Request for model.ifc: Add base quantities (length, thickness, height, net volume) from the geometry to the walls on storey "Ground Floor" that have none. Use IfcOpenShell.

First a look at what the model holds.

```python
import ifcopenshell
import ifcopenshell.util.element
import ifcopenshell.util.unit

model = ifcopenshell.open("model.ifc")
print(model.schema)
for unit_type in ("LENGTHUNIT", "AREAUNIT", "VOLUMEUNIT"):
    print(unit_type, ifcopenshell.util.unit.calculate_unit_scale(model, unit_type))
storey = next(s for s in model.by_type("IfcBuildingStorey") if s.Name == "Ground Floor")
walls = [e for e in ifcopenshell.util.element.get_decomposition(storey) if e.is_a("IfcWall")]
for e in sorted(walls, key=lambda e: e.id()):
    print(e.id(), e.is_a(), e.Name, list(ifcopenshell.util.element.get_psets(e, qtos_only=True)), sep=" | ")
```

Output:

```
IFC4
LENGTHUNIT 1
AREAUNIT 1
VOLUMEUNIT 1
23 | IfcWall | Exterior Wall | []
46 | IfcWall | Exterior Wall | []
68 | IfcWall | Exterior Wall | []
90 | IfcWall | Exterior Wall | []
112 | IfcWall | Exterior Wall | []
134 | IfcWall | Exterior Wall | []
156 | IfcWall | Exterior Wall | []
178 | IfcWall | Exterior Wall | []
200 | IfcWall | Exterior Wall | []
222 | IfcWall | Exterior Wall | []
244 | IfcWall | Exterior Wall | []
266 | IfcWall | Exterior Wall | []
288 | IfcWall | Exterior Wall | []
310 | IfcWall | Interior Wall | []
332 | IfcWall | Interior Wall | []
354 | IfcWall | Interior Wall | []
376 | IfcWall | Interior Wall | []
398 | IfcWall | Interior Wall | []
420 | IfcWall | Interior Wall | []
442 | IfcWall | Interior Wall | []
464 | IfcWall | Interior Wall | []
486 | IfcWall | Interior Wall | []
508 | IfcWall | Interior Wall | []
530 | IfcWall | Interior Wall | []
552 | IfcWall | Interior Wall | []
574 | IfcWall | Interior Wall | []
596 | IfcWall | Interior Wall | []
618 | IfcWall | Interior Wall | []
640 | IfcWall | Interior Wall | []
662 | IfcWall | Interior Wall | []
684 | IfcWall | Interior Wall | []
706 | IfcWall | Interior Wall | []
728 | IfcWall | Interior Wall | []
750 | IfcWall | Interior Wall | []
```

```python
import ifcopenshell
import ifcopenshell.api.pset
import ifcopenshell.geom
import ifcopenshell.util.element
import ifcopenshell.util.shape
import ifcopenshell.util.unit

model = ifcopenshell.open("model.ifc")
unit_scale = ifcopenshell.util.unit.calculate_unit_scale(model)
volume_scale = ifcopenshell.util.unit.calculate_unit_scale(model, "VOLUMEUNIT")
settings = ifcopenshell.geom.settings()

storey = next(s for s in model.by_type("IfcBuildingStorey") if s.Name == "Ground Floor")
walls = [e for e in ifcopenshell.util.element.get_decomposition(storey) if e.is_a("IfcWall")]

for e in sorted(walls, key=lambda e: e.id()):
    if ifcopenshell.util.element.get_psets(e, qtos_only=True, should_inherit=False):
        continue
    # Geometry comes back in metres, in the element's own axes.
    shape = ifcopenshell.geom.create_shape(settings, e)
    values = {
        "Length": ifcopenshell.util.shape.get_x(shape.geometry) / unit_scale,
        "Width": ifcopenshell.util.shape.get_y(shape.geometry) / unit_scale,
        "Height": ifcopenshell.util.shape.get_z(shape.geometry) / unit_scale,
        "NetVolume": ifcopenshell.util.shape.get_volume(shape.geometry) / volume_scale,
    }
    qto = ifcopenshell.api.pset.add_qto(model, product=e, name="Qto_WallBaseQuantities")
    ifcopenshell.api.pset.edit_qto(model, qto=qto, properties=values)
    print(e.id(), {k: round(v, 3) for k, v in values.items()})

model.write("model_v2.ifc")
```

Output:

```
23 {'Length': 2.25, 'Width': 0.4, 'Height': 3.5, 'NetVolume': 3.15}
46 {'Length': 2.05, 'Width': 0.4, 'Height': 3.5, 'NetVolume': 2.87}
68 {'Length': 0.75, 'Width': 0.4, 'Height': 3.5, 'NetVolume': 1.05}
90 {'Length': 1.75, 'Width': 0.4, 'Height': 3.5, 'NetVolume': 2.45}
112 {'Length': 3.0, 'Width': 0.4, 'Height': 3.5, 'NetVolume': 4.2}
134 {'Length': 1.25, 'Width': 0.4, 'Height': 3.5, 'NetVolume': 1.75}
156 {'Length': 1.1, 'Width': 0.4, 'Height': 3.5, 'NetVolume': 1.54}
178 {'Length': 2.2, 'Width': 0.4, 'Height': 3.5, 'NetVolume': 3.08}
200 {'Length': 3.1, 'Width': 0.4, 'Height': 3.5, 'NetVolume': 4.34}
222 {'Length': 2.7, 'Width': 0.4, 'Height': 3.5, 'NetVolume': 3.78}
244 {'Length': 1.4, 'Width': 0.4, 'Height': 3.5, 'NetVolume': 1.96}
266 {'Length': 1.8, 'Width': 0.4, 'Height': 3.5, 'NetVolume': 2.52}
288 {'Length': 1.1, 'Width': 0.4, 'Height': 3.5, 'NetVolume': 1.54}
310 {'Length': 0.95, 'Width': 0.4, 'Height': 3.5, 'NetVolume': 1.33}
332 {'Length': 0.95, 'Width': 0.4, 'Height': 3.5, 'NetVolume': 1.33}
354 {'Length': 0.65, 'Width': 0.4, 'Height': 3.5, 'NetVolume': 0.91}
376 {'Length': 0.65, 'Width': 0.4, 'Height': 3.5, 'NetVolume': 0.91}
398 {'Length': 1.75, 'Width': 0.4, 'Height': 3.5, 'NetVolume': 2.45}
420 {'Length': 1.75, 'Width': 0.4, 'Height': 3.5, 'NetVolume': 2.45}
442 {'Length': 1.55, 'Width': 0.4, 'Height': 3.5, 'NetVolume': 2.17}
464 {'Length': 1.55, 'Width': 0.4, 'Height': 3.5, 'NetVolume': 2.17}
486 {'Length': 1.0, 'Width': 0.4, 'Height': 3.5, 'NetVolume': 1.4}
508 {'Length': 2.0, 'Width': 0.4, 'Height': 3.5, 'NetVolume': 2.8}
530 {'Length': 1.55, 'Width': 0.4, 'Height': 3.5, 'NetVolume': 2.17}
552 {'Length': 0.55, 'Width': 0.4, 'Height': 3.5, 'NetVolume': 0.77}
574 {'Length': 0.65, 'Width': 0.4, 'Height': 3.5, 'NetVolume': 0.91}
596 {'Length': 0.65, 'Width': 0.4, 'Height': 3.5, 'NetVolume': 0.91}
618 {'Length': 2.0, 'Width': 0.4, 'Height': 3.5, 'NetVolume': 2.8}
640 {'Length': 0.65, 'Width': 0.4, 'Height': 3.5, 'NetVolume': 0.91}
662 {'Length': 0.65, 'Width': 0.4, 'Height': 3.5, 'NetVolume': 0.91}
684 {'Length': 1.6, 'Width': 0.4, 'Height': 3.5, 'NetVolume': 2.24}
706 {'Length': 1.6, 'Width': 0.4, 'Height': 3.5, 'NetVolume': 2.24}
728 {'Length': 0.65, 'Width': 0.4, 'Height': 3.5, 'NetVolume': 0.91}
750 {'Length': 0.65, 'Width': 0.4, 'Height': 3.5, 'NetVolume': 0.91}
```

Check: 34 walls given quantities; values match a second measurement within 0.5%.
